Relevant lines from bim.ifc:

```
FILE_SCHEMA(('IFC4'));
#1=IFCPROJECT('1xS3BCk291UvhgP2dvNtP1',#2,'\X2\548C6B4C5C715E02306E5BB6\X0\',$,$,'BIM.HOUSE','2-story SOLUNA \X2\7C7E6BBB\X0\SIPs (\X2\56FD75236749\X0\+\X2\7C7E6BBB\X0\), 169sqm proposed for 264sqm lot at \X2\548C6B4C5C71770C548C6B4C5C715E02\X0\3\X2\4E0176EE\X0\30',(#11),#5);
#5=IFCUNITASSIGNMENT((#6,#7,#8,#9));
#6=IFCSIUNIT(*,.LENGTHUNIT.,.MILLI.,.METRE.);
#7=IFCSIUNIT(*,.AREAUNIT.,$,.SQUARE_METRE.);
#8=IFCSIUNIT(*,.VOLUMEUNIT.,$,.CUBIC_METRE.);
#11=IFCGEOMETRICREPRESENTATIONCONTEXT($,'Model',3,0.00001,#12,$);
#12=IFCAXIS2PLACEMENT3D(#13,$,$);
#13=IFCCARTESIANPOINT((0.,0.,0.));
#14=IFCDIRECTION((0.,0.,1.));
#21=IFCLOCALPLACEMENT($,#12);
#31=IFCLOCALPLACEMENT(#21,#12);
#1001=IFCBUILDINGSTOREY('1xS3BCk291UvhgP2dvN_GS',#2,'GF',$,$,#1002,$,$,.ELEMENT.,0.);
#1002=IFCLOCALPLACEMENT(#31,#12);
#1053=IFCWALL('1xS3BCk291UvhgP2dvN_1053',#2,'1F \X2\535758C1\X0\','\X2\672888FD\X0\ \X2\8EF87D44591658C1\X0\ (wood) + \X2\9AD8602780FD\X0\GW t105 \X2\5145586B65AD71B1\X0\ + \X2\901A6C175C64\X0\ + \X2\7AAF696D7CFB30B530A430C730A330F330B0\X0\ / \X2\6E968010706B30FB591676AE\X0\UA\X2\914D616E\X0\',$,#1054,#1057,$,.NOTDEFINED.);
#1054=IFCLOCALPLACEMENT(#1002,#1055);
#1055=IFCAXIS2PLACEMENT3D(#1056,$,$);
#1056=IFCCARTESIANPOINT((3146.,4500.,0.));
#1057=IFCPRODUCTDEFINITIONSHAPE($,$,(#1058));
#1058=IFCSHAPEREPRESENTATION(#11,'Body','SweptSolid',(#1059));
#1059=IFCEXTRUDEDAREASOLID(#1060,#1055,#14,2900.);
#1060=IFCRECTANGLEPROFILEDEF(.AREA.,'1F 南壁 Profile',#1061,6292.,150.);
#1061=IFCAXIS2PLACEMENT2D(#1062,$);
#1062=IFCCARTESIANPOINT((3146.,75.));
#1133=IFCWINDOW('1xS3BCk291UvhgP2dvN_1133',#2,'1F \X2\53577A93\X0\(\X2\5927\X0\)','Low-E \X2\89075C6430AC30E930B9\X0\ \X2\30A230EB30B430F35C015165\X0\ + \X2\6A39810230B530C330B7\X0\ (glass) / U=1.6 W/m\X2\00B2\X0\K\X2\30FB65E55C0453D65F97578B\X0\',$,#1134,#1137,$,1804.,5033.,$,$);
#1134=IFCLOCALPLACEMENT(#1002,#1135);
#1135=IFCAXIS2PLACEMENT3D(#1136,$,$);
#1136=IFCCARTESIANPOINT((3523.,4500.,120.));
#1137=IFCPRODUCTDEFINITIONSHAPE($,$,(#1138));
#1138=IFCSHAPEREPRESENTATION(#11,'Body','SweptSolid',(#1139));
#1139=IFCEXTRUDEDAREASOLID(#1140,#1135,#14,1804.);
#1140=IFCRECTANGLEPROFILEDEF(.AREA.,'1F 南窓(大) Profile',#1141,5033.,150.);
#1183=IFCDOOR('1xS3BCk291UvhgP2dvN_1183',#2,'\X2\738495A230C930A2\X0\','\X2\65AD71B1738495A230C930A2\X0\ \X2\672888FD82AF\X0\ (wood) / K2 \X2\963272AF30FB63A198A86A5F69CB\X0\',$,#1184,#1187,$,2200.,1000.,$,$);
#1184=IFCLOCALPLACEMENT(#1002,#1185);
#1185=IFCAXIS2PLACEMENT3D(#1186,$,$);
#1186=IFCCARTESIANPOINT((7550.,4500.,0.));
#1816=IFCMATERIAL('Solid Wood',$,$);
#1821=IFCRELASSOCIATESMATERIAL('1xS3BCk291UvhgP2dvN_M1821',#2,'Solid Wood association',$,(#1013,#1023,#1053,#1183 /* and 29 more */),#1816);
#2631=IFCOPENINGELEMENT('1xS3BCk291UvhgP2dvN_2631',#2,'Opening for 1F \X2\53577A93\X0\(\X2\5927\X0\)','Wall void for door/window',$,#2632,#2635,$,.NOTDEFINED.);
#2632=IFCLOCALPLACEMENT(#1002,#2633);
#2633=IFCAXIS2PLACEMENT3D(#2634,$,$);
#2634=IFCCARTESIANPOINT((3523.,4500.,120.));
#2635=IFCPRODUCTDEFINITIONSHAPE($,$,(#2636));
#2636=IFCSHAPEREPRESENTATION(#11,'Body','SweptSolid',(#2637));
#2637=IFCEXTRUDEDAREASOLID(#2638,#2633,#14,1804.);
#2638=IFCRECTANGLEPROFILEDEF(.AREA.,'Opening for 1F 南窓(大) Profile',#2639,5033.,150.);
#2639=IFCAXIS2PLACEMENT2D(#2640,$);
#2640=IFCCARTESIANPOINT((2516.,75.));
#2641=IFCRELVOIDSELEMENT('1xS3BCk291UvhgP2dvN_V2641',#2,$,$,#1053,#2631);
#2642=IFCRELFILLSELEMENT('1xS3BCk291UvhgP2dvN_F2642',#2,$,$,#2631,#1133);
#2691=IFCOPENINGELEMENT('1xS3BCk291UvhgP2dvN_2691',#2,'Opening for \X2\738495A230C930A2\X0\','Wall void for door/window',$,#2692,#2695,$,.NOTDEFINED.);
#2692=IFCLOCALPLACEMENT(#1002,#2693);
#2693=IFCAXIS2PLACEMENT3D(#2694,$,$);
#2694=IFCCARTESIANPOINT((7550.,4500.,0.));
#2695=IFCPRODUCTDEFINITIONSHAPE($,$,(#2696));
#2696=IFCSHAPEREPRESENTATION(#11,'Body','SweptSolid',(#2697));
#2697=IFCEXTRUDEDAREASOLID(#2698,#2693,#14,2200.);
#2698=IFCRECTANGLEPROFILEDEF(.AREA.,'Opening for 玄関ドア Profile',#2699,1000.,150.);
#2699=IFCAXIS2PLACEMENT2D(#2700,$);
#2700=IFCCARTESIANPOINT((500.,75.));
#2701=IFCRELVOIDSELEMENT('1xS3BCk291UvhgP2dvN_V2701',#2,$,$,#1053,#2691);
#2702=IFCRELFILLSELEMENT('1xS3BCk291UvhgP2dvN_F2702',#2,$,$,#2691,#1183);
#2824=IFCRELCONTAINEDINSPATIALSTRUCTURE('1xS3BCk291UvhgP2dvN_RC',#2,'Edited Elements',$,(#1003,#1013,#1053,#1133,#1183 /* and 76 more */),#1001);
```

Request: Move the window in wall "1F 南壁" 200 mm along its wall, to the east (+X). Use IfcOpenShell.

```python
import ifcopenshell
import ifcopenshell.api.geometry
import ifcopenshell.util.placement
import ifcopenshell.util.unit

model = ifcopenshell.open("bim.ifc")
unit_scale = ifcopenshell.util.unit.calculate_unit_scale(model)

window = model.by_guid("1xS3BCk291UvhgP2dvN_1133")
opening = window.FillsVoids[0].RelatingOpeningElement
wall = opening.VoidsElements[0].RelatingBuildingElement

wall_matrix = ifcopenshell.util.placement.get_local_placement(wall.ObjectPlacement)
shift = wall_matrix[:3, 0] * 0.2 / unit_scale
before = ifcopenshell.util.placement.get_local_placement(window.ObjectPlacement)[:3, 3].copy()

# The window is not placed relative to its opening, so move both.
for product in (opening, window):
    matrix = ifcopenshell.util.placement.get_local_placement(product.ObjectPlacement)
    matrix[:3, 3] += shift
    ifcopenshell.api.geometry.edit_object_placement(model, product=product, matrix=matrix, is_si=False)

after = ifcopenshell.util.placement.get_local_placement(window.ObjectPlacement)[:3, 3]
print("window moved by", (after - before).round(3) + 0.0)

model.write("bim_rev.ifc")
```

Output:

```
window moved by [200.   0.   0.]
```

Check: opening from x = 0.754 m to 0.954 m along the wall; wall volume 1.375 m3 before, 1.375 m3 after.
